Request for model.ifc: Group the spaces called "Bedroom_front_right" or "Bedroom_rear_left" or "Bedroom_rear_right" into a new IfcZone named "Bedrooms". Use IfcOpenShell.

First a look at what the model holds.

```python
import ifcopenshell

model = ifcopenshell.open("model.ifc")
print(model.schema)
seen = {}
for space in model.by_type("IfcSpace"):
    seen[space.LongName] = seen.get(space.LongName, 0) + 1
for name, count in sorted(seen.items(), key=str):
    print(count, "x", name)
print("zones:", [z.Name for z in model.by_type("IfcZone")][:20])
```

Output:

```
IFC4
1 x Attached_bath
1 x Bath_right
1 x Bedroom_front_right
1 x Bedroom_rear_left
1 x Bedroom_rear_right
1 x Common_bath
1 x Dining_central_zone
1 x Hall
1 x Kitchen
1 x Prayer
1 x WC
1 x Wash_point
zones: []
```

```python
import ifcopenshell
import ifcopenshell.api.group
import ifcopenshell.api.root

model = ifcopenshell.open("model.ifc")

names = {"Bedroom_front_right", "Bedroom_rear_left", "Bedroom_rear_right"}
spaces = [s for s in model.by_type("IfcSpace") if s.LongName in names]

zone = ifcopenshell.api.root.create_entity(model, ifc_class="IfcZone", name="Bedrooms")
ifcopenshell.api.group.assign_group(model, products=spaces, group=zone)
print(len(spaces), "spaces in", zone.Name)

model.write("model_rev.ifc")
```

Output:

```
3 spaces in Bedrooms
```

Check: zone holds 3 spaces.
